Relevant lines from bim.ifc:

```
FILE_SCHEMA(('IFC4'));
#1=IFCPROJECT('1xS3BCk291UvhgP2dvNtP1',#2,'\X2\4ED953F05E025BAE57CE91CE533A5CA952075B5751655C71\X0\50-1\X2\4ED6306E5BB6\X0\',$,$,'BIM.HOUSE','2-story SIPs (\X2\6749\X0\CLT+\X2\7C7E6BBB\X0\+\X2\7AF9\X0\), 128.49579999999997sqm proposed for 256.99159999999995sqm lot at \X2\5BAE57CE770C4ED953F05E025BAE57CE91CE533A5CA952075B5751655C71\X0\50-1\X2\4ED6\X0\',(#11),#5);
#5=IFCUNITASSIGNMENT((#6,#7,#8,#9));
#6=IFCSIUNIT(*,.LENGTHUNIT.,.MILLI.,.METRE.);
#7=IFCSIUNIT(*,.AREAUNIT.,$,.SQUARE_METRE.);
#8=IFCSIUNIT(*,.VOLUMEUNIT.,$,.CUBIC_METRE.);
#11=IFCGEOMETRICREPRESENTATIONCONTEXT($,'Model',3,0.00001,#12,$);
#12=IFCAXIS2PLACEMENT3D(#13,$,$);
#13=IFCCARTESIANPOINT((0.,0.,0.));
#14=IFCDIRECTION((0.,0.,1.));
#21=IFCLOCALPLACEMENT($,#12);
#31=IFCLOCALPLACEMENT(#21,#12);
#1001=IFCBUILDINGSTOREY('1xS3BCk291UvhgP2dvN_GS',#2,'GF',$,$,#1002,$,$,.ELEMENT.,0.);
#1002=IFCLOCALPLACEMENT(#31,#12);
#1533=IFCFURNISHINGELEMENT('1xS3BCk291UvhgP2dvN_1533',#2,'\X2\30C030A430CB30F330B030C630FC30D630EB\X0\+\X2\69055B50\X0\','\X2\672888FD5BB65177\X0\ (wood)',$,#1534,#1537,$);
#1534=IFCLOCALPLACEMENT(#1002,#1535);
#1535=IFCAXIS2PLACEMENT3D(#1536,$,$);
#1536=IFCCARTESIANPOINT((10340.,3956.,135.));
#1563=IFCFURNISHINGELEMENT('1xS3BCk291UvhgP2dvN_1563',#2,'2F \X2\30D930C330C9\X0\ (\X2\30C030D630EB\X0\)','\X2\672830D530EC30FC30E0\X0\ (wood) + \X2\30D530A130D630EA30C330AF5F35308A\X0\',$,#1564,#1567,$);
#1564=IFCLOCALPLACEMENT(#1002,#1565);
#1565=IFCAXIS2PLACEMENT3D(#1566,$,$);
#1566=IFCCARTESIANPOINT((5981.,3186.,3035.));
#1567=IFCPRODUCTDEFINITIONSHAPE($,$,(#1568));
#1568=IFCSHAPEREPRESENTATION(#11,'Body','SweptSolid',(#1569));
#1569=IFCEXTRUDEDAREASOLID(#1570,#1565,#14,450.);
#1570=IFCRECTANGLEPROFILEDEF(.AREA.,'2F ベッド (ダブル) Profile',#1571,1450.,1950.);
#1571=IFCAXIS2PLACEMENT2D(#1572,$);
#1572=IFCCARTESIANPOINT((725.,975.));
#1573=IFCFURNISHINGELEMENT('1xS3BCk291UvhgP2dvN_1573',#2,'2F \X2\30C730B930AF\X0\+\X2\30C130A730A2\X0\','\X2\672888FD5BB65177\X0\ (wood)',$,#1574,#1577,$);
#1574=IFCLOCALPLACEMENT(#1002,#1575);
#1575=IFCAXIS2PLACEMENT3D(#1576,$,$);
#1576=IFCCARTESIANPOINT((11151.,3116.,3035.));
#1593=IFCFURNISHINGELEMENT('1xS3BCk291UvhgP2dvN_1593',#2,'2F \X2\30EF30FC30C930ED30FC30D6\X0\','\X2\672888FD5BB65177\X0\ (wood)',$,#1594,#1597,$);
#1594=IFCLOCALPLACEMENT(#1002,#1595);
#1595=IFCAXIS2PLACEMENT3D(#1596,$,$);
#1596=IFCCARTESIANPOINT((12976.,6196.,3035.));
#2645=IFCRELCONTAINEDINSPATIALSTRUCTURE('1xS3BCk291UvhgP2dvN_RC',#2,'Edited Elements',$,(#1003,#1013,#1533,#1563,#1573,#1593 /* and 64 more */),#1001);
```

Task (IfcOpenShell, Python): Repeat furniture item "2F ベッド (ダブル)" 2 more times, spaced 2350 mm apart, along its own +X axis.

```python
import ifcopenshell
import ifcopenshell.api.geometry
import ifcopenshell.api.root
import ifcopenshell.util.element
import ifcopenshell.util.placement

model = ifcopenshell.open("bim.ifc")


def reuse_history(source, copy):
    """copy_class also copies each property set's owner history, people and application; keep the originals."""
    for rel in copy.IsDefinedBy:
        if rel.is_a("IfcRelDefinesByProperties") and (history := rel.RelatingPropertyDefinition.OwnerHistory):
            rel.RelatingPropertyDefinition.OwnerHistory = source.OwnerHistory
            ifcopenshell.util.element.remove_deep2(model, history)


source = model.by_id(1563)
base = ifcopenshell.util.placement.get_local_placement(source.ObjectPlacement)
step = base[:3, 0] * 2350.0

for i in range(1, 3):
    copy = ifcopenshell.api.root.copy_class(model, product=source)
    copy.Representation = ifcopenshell.util.element.copy_deep(
        model, source.Representation, exclude=["IfcGeometricRepresentationContext", "IfcRepresentationMap"]
    )
    reuse_history(source, copy)
    matrix = base.copy()
    matrix[:3, 3] += i * step
    print("added at", matrix[:3, 3].round(3) + 0.0)
    ifcopenshell.api.geometry.edit_object_placement(model, product=copy, matrix=matrix, is_si=False)

model.write("bim_rev.ifc")
```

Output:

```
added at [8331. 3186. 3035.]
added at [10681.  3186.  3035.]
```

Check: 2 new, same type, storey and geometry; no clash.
